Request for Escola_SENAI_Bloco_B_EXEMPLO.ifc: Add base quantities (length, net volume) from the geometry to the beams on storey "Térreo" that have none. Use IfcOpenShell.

First a look at what the model holds.

```python
import ifcopenshell
import ifcopenshell.util.element
import ifcopenshell.util.unit

model = ifcopenshell.open("Escola_SENAI_Bloco_B_EXEMPLO.ifc")
print(model.schema)
for unit_type in ("LENGTHUNIT", "AREAUNIT", "VOLUMEUNIT"):
    print(unit_type, ifcopenshell.util.unit.calculate_unit_scale(model, unit_type))
storey = next(s for s in model.by_type("IfcBuildingStorey") if s.Name == "Térreo")
beams = [e for e in ifcopenshell.util.element.get_decomposition(storey) if e.is_a("IfcBeam")]
for e in sorted(beams, key=lambda e: e.id()):
    print(e.id(), e.is_a(), e.Name, list(ifcopenshell.util.element.get_psets(e, qtos_only=True)), sep=" | ")
```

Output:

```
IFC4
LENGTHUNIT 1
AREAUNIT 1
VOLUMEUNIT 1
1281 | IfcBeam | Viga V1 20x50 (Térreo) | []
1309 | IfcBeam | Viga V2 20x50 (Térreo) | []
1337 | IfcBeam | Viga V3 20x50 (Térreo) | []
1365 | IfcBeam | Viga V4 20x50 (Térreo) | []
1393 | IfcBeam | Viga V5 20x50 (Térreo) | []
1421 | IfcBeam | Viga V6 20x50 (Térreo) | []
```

```python
import ifcopenshell
import ifcopenshell.api.pset
import ifcopenshell.geom
import ifcopenshell.util.element
import ifcopenshell.util.shape
import ifcopenshell.util.unit

model = ifcopenshell.open("Escola_SENAI_Bloco_B_EXEMPLO.ifc")
unit_scale = ifcopenshell.util.unit.calculate_unit_scale(model)
volume_scale = ifcopenshell.util.unit.calculate_unit_scale(model, "VOLUMEUNIT")
settings = ifcopenshell.geom.settings()

storey = next(s for s in model.by_type("IfcBuildingStorey") if s.Name == "Térreo")
beams = [e for e in ifcopenshell.util.element.get_decomposition(storey) if e.is_a("IfcBeam")]

for e in sorted(beams, key=lambda e: e.id()):
    if ifcopenshell.util.element.get_psets(e, qtos_only=True, should_inherit=False):
        continue
    # Geometry comes back in metres, in the element's own axes.
    shape = ifcopenshell.geom.create_shape(settings, e)
    values = {
        "Length": ifcopenshell.util.shape.get_max_xyz(shape.geometry) / unit_scale,
        "NetVolume": ifcopenshell.util.shape.get_volume(shape.geometry) / volume_scale,
    }
    qto = ifcopenshell.api.pset.add_qto(model, product=e, name="Qto_BeamBaseQuantities")
    ifcopenshell.api.pset.edit_qto(model, qto=qto, properties=values)
    print(e.id(), {k: round(v, 3) for k, v in values.items()})

model.write("Escola_SENAI_Bloco_B_EXEMPLO_updated.ifc")
```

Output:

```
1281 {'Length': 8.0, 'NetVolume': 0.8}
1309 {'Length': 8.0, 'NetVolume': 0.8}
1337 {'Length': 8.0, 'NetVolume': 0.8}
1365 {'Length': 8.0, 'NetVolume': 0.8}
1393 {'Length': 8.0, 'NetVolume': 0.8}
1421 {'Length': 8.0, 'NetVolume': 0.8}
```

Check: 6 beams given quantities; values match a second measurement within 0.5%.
